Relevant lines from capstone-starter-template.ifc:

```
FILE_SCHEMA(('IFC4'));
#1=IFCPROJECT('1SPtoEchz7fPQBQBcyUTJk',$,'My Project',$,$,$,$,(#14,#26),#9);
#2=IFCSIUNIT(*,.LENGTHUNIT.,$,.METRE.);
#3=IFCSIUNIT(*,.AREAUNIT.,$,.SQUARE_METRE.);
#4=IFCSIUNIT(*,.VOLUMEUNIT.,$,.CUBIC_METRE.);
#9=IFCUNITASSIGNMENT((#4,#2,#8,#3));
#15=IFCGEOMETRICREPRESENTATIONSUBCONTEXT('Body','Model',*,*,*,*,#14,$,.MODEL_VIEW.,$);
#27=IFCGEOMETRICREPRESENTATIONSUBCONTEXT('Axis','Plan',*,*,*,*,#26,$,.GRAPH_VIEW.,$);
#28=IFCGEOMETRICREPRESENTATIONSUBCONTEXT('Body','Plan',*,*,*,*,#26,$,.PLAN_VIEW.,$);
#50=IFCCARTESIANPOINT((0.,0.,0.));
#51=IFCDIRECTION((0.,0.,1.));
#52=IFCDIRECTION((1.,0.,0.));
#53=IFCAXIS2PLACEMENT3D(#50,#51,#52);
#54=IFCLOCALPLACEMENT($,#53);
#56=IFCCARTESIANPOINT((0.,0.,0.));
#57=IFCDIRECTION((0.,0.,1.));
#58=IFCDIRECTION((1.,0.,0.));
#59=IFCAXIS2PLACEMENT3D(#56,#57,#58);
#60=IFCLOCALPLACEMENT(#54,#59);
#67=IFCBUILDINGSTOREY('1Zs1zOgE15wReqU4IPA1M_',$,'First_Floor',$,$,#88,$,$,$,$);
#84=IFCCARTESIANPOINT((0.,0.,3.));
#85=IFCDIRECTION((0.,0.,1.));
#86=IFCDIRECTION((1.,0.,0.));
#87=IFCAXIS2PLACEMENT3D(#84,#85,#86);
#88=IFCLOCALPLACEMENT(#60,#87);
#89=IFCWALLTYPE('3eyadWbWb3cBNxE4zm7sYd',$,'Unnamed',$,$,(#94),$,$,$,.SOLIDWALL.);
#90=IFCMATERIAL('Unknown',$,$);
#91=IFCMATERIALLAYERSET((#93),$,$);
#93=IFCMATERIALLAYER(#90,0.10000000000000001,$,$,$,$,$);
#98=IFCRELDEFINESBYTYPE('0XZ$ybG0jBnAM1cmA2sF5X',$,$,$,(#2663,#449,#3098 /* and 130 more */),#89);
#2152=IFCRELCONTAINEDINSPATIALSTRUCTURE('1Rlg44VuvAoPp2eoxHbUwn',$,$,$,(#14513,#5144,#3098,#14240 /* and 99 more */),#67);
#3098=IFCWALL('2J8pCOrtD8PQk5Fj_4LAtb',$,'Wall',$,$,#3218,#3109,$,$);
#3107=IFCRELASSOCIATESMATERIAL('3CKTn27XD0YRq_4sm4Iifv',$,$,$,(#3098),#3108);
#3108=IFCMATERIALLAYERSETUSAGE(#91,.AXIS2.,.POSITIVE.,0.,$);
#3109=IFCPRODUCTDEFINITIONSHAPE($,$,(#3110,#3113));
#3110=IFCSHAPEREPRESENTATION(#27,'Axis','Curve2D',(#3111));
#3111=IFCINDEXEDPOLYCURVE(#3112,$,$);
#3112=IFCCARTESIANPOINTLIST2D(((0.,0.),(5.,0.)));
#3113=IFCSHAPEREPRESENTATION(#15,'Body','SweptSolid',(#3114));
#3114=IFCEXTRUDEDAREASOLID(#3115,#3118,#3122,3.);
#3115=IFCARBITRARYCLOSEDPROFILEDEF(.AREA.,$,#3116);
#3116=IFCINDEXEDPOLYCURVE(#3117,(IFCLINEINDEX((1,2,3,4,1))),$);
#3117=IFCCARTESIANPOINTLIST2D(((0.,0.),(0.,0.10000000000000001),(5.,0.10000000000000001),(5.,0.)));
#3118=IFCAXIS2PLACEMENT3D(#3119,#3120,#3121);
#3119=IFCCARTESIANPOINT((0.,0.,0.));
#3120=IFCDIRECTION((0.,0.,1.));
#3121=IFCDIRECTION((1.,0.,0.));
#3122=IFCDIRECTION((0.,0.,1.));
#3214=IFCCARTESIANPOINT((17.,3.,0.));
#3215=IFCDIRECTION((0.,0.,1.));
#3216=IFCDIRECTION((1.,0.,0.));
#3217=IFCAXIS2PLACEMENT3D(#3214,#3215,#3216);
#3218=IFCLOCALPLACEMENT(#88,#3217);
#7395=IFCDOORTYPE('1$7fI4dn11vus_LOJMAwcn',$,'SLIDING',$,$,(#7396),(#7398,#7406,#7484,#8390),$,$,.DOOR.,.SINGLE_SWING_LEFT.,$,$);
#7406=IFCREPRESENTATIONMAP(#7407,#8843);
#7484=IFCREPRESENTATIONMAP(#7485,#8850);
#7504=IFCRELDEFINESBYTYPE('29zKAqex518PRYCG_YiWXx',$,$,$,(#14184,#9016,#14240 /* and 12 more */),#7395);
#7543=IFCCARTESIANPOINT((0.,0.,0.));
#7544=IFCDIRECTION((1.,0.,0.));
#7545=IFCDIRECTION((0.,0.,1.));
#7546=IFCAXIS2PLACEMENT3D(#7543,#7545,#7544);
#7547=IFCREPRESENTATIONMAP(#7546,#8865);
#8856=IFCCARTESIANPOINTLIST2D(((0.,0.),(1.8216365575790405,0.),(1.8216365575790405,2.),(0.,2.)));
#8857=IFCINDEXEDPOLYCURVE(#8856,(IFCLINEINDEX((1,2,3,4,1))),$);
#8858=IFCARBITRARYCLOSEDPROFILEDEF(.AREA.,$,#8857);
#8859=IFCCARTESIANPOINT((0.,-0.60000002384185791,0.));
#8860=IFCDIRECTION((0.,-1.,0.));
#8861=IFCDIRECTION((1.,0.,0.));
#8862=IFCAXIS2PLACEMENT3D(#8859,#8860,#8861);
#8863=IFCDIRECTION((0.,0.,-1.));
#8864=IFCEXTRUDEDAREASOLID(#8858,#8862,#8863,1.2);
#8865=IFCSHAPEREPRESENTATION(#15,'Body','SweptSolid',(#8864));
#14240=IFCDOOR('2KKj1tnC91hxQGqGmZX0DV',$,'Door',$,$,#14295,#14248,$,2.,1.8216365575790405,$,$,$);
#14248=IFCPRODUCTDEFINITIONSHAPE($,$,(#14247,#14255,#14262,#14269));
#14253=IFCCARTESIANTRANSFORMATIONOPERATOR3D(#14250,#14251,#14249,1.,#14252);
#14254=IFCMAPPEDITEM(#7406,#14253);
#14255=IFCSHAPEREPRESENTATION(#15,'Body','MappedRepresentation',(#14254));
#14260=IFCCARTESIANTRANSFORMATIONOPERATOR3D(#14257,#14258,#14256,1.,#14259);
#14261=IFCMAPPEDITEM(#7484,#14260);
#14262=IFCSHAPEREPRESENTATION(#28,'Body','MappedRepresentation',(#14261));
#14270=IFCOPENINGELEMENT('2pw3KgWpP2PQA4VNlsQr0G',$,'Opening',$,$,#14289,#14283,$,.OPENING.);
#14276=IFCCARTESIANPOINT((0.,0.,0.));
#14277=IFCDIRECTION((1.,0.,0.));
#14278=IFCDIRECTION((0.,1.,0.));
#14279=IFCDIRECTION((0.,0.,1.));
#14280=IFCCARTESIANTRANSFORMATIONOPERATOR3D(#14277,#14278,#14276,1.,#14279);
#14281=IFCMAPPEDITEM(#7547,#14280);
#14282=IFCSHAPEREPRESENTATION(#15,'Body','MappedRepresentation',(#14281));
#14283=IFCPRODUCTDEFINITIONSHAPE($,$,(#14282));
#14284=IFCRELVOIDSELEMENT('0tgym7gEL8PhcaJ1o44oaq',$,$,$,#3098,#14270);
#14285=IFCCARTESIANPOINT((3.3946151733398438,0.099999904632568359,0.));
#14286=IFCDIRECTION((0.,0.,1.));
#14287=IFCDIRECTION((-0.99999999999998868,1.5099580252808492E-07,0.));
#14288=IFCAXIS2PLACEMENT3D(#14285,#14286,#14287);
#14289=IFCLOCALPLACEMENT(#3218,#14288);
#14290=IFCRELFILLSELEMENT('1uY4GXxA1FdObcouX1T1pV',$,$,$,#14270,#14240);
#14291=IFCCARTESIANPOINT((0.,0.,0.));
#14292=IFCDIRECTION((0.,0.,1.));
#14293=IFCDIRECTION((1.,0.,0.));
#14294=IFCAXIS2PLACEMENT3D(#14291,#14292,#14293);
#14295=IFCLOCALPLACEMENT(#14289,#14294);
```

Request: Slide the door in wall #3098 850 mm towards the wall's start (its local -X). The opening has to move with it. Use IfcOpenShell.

```python
import ifcopenshell
import ifcopenshell.api.geometry
import ifcopenshell.util.placement
import ifcopenshell.util.unit

model = ifcopenshell.open("capstone-starter-template.ifc")
unit_scale = ifcopenshell.util.unit.calculate_unit_scale(model)

door = model.by_id(14240)
opening = door.FillsVoids[0].RelatingOpeningElement
wall = opening.VoidsElements[0].RelatingBuildingElement

wall_matrix = ifcopenshell.util.placement.get_local_placement(wall.ObjectPlacement)
shift = wall_matrix[:3, 0] * -0.85 / unit_scale
before = ifcopenshell.util.placement.get_local_placement(door.ObjectPlacement)[:3, 3].copy()

# The door is placed relative to its opening, so it follows when the opening moves.
matrix = ifcopenshell.util.placement.get_local_placement(opening.ObjectPlacement)
matrix[:3, 3] += shift
ifcopenshell.api.geometry.edit_object_placement(
    model, product=opening, matrix=matrix, is_si=False, should_transform_children=True
)

after = ifcopenshell.util.placement.get_local_placement(door.ObjectPlacement)[:3, 3]
print("door moved by", (after - before).round(3) + 0.0)

model.write("capstone-starter-template-out.ifc")
```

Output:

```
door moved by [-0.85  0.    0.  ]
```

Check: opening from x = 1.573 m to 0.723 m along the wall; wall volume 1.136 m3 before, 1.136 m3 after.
